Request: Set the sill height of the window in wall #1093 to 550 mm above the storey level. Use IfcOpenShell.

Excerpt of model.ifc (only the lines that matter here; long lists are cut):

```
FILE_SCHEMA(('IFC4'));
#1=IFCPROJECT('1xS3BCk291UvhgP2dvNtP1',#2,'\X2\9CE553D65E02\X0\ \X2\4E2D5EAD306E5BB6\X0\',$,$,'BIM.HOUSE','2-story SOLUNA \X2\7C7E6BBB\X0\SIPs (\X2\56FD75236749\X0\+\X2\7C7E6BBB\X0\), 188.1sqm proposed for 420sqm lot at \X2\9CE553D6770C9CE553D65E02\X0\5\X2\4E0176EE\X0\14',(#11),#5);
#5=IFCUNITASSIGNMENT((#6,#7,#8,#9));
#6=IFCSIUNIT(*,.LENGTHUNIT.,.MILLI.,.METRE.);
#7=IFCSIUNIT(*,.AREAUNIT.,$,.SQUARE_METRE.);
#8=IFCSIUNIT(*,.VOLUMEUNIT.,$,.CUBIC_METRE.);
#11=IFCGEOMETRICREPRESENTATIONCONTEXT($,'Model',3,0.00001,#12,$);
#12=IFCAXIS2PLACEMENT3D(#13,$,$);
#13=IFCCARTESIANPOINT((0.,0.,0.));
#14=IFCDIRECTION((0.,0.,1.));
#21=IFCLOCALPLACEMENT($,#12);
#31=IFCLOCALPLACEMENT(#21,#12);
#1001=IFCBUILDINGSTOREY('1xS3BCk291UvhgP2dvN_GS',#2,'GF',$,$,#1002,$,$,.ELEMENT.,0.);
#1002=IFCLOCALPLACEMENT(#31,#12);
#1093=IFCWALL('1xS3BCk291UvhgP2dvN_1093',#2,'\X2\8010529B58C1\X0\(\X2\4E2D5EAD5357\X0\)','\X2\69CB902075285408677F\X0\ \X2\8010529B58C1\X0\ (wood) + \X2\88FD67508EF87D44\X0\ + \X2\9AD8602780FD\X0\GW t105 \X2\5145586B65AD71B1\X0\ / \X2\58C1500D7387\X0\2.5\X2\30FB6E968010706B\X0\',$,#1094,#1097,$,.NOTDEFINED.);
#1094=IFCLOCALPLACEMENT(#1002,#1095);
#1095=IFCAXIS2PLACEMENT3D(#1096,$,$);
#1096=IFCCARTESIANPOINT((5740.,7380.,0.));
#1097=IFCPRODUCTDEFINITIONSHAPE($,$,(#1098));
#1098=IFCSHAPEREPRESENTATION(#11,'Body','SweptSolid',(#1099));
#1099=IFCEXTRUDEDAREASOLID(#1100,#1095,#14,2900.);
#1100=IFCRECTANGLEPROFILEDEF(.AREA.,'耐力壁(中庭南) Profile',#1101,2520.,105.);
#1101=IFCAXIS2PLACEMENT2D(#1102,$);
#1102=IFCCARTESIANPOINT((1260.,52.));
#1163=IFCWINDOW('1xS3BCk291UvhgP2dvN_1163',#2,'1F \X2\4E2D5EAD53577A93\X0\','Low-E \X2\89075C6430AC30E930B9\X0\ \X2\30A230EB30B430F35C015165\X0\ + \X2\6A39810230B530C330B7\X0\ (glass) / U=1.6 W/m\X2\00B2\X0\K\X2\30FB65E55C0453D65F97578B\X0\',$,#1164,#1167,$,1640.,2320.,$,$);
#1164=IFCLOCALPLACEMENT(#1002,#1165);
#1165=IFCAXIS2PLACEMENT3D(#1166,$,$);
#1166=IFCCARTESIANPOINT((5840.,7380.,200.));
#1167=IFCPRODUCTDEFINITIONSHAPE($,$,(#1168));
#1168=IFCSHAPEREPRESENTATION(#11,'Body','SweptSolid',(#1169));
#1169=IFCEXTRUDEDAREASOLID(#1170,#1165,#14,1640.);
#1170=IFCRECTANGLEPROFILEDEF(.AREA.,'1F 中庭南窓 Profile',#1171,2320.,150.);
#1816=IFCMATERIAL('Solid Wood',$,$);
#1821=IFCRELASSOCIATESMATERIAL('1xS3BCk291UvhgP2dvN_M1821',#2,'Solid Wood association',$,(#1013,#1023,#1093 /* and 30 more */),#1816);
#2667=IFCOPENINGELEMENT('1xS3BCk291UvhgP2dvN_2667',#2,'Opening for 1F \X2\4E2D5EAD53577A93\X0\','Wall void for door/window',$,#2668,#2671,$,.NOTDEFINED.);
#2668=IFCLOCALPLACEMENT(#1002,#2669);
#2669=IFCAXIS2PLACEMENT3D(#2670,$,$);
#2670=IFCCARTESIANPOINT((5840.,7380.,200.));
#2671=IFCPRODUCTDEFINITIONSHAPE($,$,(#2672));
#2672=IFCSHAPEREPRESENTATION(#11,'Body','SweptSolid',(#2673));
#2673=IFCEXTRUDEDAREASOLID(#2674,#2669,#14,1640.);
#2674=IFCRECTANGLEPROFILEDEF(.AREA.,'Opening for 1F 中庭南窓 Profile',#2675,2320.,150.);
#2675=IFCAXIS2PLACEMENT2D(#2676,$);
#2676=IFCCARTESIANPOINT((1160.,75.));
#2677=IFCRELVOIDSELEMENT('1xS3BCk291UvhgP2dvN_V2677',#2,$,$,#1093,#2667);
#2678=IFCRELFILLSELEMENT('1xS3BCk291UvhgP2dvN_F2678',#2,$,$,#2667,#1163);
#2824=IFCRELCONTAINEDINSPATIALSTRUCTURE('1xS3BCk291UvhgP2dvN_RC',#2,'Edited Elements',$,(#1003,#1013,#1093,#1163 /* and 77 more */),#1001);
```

```python
import numpy as np
import ifcopenshell
import ifcopenshell.api.geometry
import ifcopenshell.geom
import ifcopenshell.util.element
import ifcopenshell.util.placement
import ifcopenshell.util.shape
import ifcopenshell.util.unit

model = ifcopenshell.open("model.ifc")
unit_scale = ifcopenshell.util.unit.calculate_unit_scale(model)

window = model.by_id(1163)
opening = window.FillsVoids[0].RelatingOpeningElement
storey = ifcopenshell.util.element.get_container(window, ifc_class="IfcBuildingStorey")
level = ifcopenshell.util.placement.get_local_placement(storey.ObjectPlacement)[2, 3]

# The opening's origin need not be at the sill, so measure its lowest point.
shape = ifcopenshell.geom.create_shape(ifcopenshell.geom.settings(), opening)
bottom = ifcopenshell.util.shape.get_shape_bottom_elevation(shape, shape.geometry) / unit_scale
dz = level + 550.0 - bottom

shift = np.array([0.0, 0.0, dz])
# The window is not placed relative to its opening, so move both.
for product in (opening, window):
    matrix = ifcopenshell.util.placement.get_local_placement(product.ObjectPlacement)
    matrix[:3, 3] += shift
    ifcopenshell.api.geometry.edit_object_placement(model, product=product, matrix=matrix, is_si=False)

print(f"moved by {dz * unit_scale:+.3f} m")

model.write("model_edited.ifc")
```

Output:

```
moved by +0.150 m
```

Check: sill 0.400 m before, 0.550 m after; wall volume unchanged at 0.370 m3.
